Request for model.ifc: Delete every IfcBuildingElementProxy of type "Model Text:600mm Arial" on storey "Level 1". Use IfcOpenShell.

First a look at what the model holds.

```python
import ifcopenshell
import ifcopenshell.util.element

model = ifcopenshell.open("model.ifc")
print(model.schema)
storey = next(s for s in model.by_type("IfcBuildingStorey") if s.Name == "Level 1")
proxies = [e for e in ifcopenshell.util.element.get_decomposition(storey) if e.is_a("IfcBuildingElementProxy")]
seen = {}
for e in proxies:
    element_type = ifcopenshell.util.element.get_type(e)
    name = element_type.Name if element_type not in (None, e) else None
    seen[name] = seen.get(name, 0) + 1
for name, count in sorted(seen.items(), key=str):
    print(count, "x", name)
```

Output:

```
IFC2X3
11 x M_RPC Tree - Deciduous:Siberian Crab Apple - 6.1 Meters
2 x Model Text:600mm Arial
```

```python
import ifcopenshell
import ifcopenshell.api.root
import ifcopenshell.util.element

model = ifcopenshell.open("model.ifc")

storey = next(s for s in model.by_type("IfcBuildingStorey") if s.Name == "Level 1")
proxies = [e for e in ifcopenshell.util.element.get_decomposition(storey) if e.is_a("IfcBuildingElementProxy")]
targets = [e for e in proxies if (t := ifcopenshell.util.element.get_type(e)) not in (None, e) and t.Name == "Model Text:600mm Arial"]

for e in targets:
    ifcopenshell.api.root.remove_product(model, product=e)
print(len(targets), "removed")

model.write("model_updated.ifc")
```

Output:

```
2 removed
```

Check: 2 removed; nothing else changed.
